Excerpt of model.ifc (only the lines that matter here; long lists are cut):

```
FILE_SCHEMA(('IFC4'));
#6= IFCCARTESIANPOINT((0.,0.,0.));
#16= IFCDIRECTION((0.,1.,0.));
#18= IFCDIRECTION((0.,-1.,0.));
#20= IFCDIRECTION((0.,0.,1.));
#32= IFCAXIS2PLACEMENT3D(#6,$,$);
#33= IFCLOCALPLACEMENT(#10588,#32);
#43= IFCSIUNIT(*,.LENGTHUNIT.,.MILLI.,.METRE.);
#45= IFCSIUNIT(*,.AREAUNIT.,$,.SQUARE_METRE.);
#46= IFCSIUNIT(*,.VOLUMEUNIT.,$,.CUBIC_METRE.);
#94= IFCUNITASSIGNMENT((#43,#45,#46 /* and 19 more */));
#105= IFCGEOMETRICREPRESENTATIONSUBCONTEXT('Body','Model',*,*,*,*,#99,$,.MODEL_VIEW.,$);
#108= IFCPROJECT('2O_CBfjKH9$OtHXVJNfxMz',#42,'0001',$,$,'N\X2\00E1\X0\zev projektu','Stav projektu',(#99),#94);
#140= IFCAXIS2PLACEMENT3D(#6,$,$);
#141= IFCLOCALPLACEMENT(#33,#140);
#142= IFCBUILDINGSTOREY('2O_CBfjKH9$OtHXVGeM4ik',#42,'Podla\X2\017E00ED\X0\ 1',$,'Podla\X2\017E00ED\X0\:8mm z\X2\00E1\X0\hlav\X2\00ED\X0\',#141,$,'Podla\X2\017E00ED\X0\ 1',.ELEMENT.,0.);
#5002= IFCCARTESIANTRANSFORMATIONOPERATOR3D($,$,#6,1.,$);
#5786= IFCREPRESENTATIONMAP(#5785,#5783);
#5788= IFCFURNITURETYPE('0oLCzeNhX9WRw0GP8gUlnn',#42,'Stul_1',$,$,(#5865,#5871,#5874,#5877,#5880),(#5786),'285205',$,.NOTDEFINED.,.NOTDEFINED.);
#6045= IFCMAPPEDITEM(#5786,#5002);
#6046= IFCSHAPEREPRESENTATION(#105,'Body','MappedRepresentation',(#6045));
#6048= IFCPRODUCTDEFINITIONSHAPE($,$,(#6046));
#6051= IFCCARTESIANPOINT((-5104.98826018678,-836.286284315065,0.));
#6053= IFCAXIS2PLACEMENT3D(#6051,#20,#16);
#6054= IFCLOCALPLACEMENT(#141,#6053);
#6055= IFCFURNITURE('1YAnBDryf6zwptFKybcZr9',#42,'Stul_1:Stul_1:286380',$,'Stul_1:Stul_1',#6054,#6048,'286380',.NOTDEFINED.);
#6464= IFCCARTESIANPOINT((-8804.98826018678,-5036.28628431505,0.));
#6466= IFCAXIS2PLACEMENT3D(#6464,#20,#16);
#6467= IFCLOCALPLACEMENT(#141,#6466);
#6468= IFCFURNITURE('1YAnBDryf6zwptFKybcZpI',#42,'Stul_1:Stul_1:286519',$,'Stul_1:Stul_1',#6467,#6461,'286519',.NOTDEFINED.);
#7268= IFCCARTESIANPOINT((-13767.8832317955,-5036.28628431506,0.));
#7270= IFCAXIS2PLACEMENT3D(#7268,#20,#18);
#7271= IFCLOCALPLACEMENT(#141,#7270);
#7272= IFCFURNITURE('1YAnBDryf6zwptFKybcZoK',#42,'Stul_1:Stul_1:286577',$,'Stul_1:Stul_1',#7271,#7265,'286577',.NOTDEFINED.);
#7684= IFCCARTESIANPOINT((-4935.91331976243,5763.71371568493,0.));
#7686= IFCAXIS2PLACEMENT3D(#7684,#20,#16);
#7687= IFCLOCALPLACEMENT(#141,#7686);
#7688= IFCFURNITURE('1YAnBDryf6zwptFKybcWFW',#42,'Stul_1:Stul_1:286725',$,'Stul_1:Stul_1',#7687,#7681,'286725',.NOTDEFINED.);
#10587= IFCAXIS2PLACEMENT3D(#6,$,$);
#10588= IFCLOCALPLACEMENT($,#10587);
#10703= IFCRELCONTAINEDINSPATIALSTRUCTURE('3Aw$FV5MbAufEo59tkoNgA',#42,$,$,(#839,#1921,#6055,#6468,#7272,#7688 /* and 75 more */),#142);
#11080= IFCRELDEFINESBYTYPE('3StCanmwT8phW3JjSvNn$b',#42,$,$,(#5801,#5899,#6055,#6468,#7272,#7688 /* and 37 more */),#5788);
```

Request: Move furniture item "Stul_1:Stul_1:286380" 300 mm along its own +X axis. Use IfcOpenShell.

```python
import ifcopenshell
import ifcopenshell.api.geometry
import ifcopenshell.util.placement

model = ifcopenshell.open("model.ifc")

item = model.by_guid("1YAnBDryf6zwptFKybcZr9")
matrix = ifcopenshell.util.placement.get_local_placement(item.ObjectPlacement)
matrix[:3, 3] += matrix[:3, 0] * 300.0
ifcopenshell.api.geometry.edit_object_placement(model, product=item, matrix=matrix, is_si=False)

print(ifcopenshell.util.placement.get_local_placement(item.ObjectPlacement).round(3) + 0.0)

model.write("model_edited.ifc")
```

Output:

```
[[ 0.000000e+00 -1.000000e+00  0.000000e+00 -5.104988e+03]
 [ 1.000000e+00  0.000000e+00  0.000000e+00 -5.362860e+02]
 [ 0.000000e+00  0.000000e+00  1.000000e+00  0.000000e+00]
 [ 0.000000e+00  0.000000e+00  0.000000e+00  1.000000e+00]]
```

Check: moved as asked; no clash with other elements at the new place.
